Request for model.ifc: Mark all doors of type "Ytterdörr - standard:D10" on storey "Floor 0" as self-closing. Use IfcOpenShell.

First a look at what the model holds.

```python
import ifcopenshell
import ifcopenshell.util.element

model = ifcopenshell.open("model.ifc")
print(model.schema)
storey = next(s for s in model.by_type("IfcBuildingStorey") if s.Name == "Floor 0")
doors = [e for e in ifcopenshell.util.element.get_decomposition(storey) if e.is_a("IfcDoor")]
seen = {}
for e in doors:
    element_type = ifcopenshell.util.element.get_type(e)
    key = (element_type.Name if element_type != e and element_type else None, ifcopenshell.util.element.get_pset(e, "Pset_DoorCommon", "SelfClosing"))
    seen[key] = seen.get(key, 0) + 1
for (name, value), count in sorted(seen.items(), key=str):
    print(count, "x", name, "|", value)
```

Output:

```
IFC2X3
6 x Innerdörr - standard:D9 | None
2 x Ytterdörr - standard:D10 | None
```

```python
import ifcopenshell
import ifcopenshell.api.pset
import ifcopenshell.util.element

model = ifcopenshell.open("model.ifc")

storey = next(s for s in model.by_type("IfcBuildingStorey") if s.Name == "Floor 0")
doors = [e for e in ifcopenshell.util.element.get_decomposition(storey) if e.is_a("IfcDoor")]

count = 0
for e in doors:
    element_type = ifcopenshell.util.element.get_type(e)
    if element_type in (None, e) or element_type.Name != "Ytterdörr - standard:D10":
        continue
    # add_pset returns the element's existing set when there is one.
    pset = ifcopenshell.api.pset.add_pset(model, product=e, name="Pset_DoorCommon")
    ifcopenshell.api.pset.edit_pset(model, pset=pset, properties={"SelfClosing": True})
    count += 1

print(count, "doors updated")

model.write("model_rev.ifc")
```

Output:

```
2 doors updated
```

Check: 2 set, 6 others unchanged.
